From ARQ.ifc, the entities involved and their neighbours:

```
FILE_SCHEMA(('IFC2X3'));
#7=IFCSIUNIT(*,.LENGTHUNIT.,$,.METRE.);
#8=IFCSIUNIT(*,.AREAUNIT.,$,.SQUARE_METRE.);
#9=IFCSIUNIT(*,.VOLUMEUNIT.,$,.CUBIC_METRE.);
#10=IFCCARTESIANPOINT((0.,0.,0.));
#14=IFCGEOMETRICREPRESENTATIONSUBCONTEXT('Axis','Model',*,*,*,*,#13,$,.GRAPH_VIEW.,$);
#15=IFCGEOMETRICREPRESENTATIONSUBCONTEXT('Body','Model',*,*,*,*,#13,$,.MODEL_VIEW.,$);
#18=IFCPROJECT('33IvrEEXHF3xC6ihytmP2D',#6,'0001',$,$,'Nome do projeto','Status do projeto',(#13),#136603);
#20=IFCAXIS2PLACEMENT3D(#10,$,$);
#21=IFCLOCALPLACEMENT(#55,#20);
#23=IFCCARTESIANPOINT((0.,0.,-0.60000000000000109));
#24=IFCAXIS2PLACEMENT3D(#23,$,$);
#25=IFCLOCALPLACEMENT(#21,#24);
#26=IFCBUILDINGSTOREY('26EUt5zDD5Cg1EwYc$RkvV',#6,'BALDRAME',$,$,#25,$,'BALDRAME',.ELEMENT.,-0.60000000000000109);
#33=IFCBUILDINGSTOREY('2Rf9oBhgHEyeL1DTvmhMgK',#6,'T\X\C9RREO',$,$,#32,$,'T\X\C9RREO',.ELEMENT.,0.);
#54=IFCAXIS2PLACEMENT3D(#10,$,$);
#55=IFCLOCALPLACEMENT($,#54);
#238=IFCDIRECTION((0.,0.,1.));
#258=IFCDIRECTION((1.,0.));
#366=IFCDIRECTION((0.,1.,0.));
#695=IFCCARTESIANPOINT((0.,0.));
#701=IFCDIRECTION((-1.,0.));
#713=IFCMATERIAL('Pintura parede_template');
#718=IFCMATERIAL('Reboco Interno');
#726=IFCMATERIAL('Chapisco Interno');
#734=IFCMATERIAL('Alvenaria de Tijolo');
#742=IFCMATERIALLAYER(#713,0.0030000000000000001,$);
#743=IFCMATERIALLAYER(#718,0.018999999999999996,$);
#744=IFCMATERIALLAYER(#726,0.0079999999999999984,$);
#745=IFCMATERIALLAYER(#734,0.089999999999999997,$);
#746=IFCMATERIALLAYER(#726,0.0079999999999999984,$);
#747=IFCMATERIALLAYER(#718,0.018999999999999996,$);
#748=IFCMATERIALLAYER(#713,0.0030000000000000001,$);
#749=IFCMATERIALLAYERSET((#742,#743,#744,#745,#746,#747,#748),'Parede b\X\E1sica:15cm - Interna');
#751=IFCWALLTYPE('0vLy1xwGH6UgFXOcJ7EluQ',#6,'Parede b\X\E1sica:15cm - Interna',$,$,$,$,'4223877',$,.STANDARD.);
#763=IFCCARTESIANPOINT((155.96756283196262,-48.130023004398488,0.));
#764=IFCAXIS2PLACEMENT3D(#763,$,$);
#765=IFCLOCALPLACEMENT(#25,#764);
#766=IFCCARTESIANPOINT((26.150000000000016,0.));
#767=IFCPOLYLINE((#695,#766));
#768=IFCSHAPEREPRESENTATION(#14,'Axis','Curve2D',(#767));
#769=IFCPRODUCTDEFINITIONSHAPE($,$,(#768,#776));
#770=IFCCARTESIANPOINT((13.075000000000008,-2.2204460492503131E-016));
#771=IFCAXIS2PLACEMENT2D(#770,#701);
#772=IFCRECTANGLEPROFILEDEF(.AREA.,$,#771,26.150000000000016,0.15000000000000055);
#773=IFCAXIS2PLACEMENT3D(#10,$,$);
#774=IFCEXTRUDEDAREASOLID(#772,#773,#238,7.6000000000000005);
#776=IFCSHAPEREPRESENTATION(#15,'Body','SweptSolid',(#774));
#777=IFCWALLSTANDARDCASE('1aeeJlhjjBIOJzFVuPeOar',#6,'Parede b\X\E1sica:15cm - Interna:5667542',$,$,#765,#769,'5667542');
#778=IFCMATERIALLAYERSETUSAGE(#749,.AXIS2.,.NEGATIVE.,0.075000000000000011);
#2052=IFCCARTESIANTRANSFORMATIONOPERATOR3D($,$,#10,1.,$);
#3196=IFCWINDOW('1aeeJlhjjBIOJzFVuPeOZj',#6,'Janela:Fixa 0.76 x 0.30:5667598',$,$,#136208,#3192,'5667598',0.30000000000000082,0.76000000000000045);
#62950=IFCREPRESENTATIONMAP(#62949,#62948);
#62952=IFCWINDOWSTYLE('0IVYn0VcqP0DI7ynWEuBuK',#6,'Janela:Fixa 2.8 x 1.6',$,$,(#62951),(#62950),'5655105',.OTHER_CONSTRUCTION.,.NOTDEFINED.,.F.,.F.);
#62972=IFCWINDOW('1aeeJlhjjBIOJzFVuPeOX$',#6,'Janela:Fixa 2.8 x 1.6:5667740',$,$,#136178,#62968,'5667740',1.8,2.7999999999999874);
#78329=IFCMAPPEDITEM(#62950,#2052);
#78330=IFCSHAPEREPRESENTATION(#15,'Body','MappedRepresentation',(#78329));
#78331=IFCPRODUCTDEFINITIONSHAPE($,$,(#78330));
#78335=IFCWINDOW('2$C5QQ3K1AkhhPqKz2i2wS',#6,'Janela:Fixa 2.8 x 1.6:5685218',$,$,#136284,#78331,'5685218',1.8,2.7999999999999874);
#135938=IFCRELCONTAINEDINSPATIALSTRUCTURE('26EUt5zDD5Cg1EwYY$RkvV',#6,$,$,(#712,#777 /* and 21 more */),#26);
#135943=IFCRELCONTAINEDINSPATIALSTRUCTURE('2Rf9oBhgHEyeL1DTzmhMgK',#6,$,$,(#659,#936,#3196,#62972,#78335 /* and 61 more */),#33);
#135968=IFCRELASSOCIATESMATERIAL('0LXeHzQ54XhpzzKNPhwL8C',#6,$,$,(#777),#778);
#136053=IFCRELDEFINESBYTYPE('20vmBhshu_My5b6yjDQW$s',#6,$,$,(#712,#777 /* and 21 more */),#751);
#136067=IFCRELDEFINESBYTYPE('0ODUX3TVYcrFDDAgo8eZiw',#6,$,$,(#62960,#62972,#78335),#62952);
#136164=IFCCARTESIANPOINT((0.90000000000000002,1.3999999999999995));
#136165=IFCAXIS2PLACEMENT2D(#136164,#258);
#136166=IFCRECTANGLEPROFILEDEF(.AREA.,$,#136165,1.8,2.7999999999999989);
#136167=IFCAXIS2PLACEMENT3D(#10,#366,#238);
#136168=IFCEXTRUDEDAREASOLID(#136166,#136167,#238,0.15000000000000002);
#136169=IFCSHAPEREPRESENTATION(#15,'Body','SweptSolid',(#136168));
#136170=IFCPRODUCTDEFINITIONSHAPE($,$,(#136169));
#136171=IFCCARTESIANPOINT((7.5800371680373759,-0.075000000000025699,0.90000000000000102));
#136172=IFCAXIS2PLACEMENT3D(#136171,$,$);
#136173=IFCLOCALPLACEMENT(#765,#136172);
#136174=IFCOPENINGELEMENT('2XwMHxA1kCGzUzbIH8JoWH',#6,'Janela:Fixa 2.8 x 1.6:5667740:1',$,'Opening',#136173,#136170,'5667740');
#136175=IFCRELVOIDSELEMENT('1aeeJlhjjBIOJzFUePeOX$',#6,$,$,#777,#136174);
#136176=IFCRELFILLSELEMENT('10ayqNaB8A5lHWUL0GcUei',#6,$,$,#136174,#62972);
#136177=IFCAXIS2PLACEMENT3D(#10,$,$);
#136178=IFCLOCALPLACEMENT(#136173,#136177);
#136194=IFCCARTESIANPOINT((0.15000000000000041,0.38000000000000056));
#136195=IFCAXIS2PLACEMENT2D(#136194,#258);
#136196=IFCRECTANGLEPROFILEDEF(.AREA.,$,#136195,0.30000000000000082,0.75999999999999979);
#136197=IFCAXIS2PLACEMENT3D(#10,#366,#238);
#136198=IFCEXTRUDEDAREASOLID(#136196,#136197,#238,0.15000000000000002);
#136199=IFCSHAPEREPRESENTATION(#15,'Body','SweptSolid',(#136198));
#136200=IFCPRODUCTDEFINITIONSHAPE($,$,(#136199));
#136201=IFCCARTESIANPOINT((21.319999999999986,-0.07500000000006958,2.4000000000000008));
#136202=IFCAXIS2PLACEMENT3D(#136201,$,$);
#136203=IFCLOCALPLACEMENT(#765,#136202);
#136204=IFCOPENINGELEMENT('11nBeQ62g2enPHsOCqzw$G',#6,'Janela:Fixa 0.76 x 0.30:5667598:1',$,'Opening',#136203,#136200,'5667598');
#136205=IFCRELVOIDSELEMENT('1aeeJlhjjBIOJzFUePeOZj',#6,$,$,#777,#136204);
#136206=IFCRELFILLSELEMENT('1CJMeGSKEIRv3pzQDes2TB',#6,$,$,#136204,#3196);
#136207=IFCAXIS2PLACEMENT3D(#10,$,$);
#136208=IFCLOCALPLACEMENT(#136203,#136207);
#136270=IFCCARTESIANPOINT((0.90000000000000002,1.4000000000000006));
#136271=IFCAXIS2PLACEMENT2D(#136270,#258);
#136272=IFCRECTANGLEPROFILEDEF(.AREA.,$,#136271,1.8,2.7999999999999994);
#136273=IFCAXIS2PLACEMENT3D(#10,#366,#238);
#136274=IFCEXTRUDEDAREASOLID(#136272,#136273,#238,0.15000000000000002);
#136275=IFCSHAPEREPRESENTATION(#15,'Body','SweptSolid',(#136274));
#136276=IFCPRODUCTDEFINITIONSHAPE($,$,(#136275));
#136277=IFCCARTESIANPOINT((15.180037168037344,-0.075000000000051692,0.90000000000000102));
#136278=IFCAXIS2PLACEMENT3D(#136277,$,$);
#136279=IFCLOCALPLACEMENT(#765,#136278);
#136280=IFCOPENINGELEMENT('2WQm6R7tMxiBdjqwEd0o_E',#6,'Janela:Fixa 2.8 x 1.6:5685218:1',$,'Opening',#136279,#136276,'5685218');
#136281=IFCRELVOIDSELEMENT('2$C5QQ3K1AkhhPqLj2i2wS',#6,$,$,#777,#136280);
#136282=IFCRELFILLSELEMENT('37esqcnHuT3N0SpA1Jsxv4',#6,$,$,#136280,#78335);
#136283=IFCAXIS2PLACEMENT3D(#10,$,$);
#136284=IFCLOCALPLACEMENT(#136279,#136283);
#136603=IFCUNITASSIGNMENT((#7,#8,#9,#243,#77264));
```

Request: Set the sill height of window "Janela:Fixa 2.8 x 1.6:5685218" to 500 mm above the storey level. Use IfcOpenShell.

```python
import numpy as np
import ifcopenshell
import ifcopenshell.api.geometry
import ifcopenshell.geom
import ifcopenshell.util.element
import ifcopenshell.util.placement
import ifcopenshell.util.shape
import ifcopenshell.util.unit

model = ifcopenshell.open("ARQ.ifc")
unit_scale = ifcopenshell.util.unit.calculate_unit_scale(model)

window = model.by_guid("2$C5QQ3K1AkhhPqKz2i2wS")
opening = window.FillsVoids[0].RelatingOpeningElement
storey = ifcopenshell.util.element.get_container(window, ifc_class="IfcBuildingStorey")
level = ifcopenshell.util.placement.get_local_placement(storey.ObjectPlacement)[2, 3]

# The opening's origin need not be at the sill, so measure its lowest point.
shape = ifcopenshell.geom.create_shape(ifcopenshell.geom.settings(), opening)
bottom = ifcopenshell.util.shape.get_shape_bottom_elevation(shape, shape.geometry) / unit_scale
dz = level + 0.5 / unit_scale - bottom

shift = np.array([0.0, 0.0, dz])
# The window is placed relative to its opening, so it follows when the opening moves.
matrix = ifcopenshell.util.placement.get_local_placement(opening.ObjectPlacement)
matrix[:3, 3] += shift
ifcopenshell.api.geometry.edit_object_placement(
    model, product=opening, matrix=matrix, is_si=False, should_transform_children=True
)

print(f"moved by {dz * unit_scale:+.3f} m")

model.write("ARQ_updated.ifc")
```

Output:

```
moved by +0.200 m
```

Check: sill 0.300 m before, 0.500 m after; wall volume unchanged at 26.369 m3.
